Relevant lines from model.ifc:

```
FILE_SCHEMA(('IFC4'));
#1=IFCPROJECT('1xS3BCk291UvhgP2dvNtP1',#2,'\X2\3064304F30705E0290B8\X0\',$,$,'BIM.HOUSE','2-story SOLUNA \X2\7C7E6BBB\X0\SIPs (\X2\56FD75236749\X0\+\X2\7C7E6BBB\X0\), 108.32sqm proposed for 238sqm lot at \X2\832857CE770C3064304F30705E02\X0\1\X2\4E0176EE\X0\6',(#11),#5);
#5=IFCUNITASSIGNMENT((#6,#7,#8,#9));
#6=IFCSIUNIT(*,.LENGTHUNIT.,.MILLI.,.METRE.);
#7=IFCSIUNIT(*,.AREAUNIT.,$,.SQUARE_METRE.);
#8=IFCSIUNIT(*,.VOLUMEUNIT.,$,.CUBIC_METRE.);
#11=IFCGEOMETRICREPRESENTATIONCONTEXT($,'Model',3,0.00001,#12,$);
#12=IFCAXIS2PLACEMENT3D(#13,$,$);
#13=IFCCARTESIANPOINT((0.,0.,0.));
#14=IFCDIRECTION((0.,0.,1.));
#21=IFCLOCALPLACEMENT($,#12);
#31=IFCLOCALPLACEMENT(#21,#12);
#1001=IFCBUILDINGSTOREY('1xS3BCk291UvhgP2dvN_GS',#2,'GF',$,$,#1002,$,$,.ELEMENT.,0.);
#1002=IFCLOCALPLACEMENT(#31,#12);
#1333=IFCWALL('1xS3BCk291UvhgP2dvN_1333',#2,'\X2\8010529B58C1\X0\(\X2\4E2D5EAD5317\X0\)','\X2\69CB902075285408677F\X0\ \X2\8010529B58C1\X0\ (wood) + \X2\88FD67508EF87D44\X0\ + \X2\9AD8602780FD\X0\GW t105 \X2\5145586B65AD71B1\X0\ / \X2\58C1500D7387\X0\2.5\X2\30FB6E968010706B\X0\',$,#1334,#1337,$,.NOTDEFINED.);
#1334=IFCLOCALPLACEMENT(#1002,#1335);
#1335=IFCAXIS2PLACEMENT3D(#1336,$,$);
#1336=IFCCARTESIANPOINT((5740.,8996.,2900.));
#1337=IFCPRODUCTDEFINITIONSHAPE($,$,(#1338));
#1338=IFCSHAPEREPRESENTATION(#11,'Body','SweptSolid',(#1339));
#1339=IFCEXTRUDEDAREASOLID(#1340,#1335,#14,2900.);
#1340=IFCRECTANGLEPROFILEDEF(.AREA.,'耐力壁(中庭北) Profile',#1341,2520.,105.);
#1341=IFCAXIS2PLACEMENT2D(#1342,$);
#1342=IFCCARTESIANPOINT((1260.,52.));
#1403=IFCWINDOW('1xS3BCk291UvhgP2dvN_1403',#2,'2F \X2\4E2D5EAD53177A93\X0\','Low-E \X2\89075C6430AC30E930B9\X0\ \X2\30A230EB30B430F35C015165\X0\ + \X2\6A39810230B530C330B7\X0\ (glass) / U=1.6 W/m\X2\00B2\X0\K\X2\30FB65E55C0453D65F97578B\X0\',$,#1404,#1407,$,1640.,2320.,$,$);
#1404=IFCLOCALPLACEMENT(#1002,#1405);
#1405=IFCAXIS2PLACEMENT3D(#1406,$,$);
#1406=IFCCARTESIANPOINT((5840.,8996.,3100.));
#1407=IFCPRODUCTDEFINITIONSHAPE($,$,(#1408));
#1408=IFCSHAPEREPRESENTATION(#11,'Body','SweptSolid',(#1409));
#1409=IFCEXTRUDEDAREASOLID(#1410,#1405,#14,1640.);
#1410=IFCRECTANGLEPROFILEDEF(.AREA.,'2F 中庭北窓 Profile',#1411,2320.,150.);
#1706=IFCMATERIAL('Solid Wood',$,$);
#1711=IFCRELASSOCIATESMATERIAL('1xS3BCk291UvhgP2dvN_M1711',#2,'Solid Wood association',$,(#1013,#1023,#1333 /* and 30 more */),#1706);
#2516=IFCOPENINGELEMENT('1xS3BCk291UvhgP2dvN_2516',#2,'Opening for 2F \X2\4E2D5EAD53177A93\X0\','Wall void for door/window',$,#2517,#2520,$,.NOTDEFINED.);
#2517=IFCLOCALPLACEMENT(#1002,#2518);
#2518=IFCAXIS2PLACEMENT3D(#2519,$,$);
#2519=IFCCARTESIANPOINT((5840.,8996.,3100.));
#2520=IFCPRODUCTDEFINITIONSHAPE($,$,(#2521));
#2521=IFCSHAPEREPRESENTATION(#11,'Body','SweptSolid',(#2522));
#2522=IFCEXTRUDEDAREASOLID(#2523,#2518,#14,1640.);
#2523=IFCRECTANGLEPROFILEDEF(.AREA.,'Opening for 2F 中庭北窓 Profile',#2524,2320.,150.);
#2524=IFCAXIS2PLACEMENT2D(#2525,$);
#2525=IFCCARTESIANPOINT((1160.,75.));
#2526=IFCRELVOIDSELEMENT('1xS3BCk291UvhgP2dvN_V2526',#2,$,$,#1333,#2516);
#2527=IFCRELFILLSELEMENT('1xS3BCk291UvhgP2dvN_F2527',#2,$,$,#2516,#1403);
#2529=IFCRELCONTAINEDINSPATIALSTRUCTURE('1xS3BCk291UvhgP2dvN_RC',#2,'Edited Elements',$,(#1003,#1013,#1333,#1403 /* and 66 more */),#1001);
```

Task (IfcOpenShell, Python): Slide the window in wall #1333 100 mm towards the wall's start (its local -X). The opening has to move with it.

```python
import ifcopenshell
import ifcopenshell.api.geometry
import ifcopenshell.util.placement
import ifcopenshell.util.unit

model = ifcopenshell.open("model.ifc")
unit_scale = ifcopenshell.util.unit.calculate_unit_scale(model)

window = model.by_guid("1xS3BCk291UvhgP2dvN_1403")
opening = window.FillsVoids[0].RelatingOpeningElement
wall = opening.VoidsElements[0].RelatingBuildingElement

wall_matrix = ifcopenshell.util.placement.get_local_placement(wall.ObjectPlacement)
shift = wall_matrix[:3, 0] * -0.1 / unit_scale
before = ifcopenshell.util.placement.get_local_placement(window.ObjectPlacement)[:3, 3].copy()

# The window is not placed relative to its opening, so move both.
for product in (opening, window):
    matrix = ifcopenshell.util.placement.get_local_placement(product.ObjectPlacement)
    matrix[:3, 3] += shift
    ifcopenshell.api.geometry.edit_object_placement(model, product=product, matrix=matrix, is_si=False)

after = ifcopenshell.util.placement.get_local_placement(window.ObjectPlacement)[:3, 3]
print("window moved by", (after - before).round(3) + 0.0)

model.write("model_rev.ifc")
```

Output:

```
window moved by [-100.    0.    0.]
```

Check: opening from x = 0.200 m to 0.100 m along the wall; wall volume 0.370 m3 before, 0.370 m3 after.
